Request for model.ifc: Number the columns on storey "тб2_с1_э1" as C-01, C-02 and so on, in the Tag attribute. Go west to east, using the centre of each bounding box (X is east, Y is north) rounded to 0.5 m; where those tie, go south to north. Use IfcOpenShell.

First a look at what the model holds.

```python
import ifcopenshell
import ifcopenshell.util.element
import ifcopenshell.util.placement

model = ifcopenshell.open("model.ifc")
print(model.schema)
storey = next(s for s in model.by_type("IfcBuildingStorey") if s.Name == "тб2_с1_э1")
columns = [e for e in ifcopenshell.util.element.get_decomposition(storey) if e.is_a("IfcColumn")]
for e in sorted(columns, key=lambda e: e.id()):
    origin = ifcopenshell.util.placement.get_local_placement(e.ObjectPlacement)[:3, 3]
    print(e.id(), e.Tag, e.Name, origin.round(2) + 0.0, sep=" | ")
```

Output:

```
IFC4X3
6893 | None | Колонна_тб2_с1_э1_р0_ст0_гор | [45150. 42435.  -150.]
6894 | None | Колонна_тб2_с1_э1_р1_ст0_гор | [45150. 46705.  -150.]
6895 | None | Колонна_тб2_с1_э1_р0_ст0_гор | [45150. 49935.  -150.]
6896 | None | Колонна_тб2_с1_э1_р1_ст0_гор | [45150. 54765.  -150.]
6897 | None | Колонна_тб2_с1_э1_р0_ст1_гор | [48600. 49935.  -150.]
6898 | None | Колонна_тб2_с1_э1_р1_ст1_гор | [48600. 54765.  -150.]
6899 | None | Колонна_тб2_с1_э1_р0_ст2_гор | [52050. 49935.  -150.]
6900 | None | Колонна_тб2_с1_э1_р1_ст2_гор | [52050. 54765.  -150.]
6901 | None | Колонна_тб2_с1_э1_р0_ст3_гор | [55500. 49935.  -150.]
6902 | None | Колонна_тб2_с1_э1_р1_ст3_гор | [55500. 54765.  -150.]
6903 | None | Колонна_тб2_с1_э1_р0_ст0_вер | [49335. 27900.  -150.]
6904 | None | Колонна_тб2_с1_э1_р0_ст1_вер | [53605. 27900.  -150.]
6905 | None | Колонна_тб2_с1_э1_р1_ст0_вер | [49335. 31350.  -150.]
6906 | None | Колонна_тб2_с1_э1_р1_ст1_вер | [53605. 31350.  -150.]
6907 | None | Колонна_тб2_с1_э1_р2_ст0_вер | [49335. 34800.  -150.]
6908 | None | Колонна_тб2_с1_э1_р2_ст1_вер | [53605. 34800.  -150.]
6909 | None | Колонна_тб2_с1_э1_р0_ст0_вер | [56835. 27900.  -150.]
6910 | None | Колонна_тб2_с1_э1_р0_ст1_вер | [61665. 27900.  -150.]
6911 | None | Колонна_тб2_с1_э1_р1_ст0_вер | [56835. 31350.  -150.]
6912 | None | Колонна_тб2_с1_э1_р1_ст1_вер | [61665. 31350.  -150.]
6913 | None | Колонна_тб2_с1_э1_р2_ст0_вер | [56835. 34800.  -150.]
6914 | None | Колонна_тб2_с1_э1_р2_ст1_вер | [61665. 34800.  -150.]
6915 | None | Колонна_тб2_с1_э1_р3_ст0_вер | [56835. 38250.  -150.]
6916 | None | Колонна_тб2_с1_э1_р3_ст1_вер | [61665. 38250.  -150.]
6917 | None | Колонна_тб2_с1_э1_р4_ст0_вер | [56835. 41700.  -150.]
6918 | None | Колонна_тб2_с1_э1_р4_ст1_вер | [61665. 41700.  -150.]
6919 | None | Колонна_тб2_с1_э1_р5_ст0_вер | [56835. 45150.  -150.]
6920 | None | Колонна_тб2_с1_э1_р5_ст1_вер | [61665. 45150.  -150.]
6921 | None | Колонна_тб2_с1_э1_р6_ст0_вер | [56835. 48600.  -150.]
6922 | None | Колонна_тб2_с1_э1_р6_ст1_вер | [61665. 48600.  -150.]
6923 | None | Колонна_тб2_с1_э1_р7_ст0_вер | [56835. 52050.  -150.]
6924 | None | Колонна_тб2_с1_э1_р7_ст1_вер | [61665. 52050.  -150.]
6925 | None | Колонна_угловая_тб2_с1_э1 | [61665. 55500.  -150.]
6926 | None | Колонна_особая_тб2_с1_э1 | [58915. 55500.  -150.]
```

```python
import ifcopenshell
import ifcopenshell.geom
import ifcopenshell.util.element
import ifcopenshell.util.shape

model = ifcopenshell.open("model.ifc")
settings = ifcopenshell.geom.settings()
settings.set("use-world-coords", True)


def centre(element):
    shape = ifcopenshell.geom.create_shape(settings, element)
    return ifcopenshell.util.shape.get_bbox_centroid(shape.geometry)


storey = next(s for s in model.by_type("IfcBuildingStorey") if s.Name == "тб2_с1_э1")
columns = [e for e in ifcopenshell.util.element.get_decomposition(storey) if e.is_a("IfcColumn")]

# Insertion points can sit at a corner or the storey origin, so sort by the geometry (in metres).
centres = {e: centre(e) for e in columns}
columns.sort(key=lambda e: (round(centres[e][0] / 0.5), centres[e][1]))

for i, e in enumerate(columns, start=1):
    number = f"C-{i:02d}"
    e.Tag = number
    print(e.id(), number)

model.write("model_v2.ifc")
```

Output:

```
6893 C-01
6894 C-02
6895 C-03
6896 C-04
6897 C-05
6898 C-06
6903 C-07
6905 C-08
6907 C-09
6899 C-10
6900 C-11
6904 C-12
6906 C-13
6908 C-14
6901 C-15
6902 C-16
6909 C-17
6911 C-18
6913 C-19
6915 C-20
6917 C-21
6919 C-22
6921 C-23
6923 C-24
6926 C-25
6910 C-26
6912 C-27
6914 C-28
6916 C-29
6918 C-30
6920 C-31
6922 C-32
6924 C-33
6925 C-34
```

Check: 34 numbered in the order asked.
